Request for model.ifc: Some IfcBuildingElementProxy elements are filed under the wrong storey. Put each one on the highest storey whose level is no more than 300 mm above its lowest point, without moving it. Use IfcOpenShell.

First a look at what the model holds.

```python
import ifcopenshell
import ifcopenshell.util.element
import ifcopenshell.util.placement

model = ifcopenshell.open("model.ifc")
print(model.schema)
for storey in model.by_type("IfcBuildingStorey"):
    level = ifcopenshell.util.placement.get_storey_elevation(storey)
    count = sum(e.is_a("IfcBuildingElementProxy") for e in ifcopenshell.util.element.get_contained(storey))
    print(storey.id(), storey.Name, round(level, 3), count, sep=" | ")
```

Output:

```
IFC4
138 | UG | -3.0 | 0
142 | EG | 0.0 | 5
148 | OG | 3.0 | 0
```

```python
import ifcopenshell
import ifcopenshell.api.spatial
import ifcopenshell.geom
import ifcopenshell.util.element
import ifcopenshell.util.placement
import ifcopenshell.util.shape
import ifcopenshell.util.unit

model = ifcopenshell.open("model.ifc")
unit_scale = ifcopenshell.util.unit.calculate_unit_scale(model)
settings = ifcopenshell.geom.settings()

levels = sorted(
    ((ifcopenshell.util.placement.get_storey_elevation(s) * unit_scale, s) for s in model.by_type("IfcBuildingStorey")),
    key=lambda pair: pair[0],
)

for e in model.by_type("IfcBuildingElementProxy"):
    current = e.ContainedInStructure[0].RelatingStructure if e.ContainedInStructure else None
    if current is None or not current.is_a("IfcBuildingStorey"):
        continue
    shape = ifcopenshell.geom.create_shape(settings, e)
    bottom = ifcopenshell.util.shape.get_shape_bottom_elevation(shape, shape.geometry)
    below = [s for level, s in levels if level <= bottom + 0.3]
    storey = below[-1] if below else levels[0][1]
    if storey != current:
        # assign_container keeps the world position.
        ifcopenshell.api.spatial.assign_container(model, products=[e], relating_structure=storey)
        print(e.id(), current.Name, "->", storey.Name)

model.write("model_edited.ifc")
```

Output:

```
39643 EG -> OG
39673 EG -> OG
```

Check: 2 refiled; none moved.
